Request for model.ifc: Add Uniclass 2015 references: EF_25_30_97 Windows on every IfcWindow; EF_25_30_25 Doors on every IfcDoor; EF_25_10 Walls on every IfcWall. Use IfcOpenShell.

First a look at what the model holds.

```python
import ifcopenshell

model = ifcopenshell.open("model.ifc")
print(model.schema)
print("classifications:", [c.Name for c in model.by_type("IfcClassification")])
for ifc_class in ("IfcDoor", "IfcRoof", "IfcStair", "IfcWall", "IfcWindow"):
    print(ifc_class, len(model.by_type(ifc_class)))
```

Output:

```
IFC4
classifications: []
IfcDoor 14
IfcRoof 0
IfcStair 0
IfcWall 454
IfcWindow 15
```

```python
import ifcopenshell
import ifcopenshell.api.classification

model = ifcopenshell.open("model.ifc")

system = ifcopenshell.api.classification.add_classification(model, classification="Uniclass 2015")

codes = {
    "IfcWindow": ("EF_25_30_97", "Windows"),
    "IfcDoor": ("EF_25_30_25", "Doors"),
    "IfcWall": ("EF_25_10", "Walls"),
}
for ifc_class, (code, name) in codes.items():
    products = model.by_type(ifc_class)
    ifcopenshell.api.classification.add_reference(
        model, products=products, classification=system, identification=code, name=name
    )
    print(code, len(products))

model.write("model_updated.ifc")
```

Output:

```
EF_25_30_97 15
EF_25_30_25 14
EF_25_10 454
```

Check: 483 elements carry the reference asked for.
